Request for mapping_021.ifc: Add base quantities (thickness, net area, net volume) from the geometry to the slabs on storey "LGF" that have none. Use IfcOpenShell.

First a look at what the model holds.

```python
import ifcopenshell
import ifcopenshell.util.element
import ifcopenshell.util.unit

model = ifcopenshell.open("mapping_021.ifc")
print(model.schema)
for unit_type in ("LENGTHUNIT", "AREAUNIT", "VOLUMEUNIT"):
    print(unit_type, ifcopenshell.util.unit.calculate_unit_scale(model, unit_type))
storey = next(s for s in model.by_type("IfcBuildingStorey") if s.Name == "LGF")
slabs = [e for e in ifcopenshell.util.element.get_decomposition(storey) if e.is_a("IfcSlab")]
for e in sorted(slabs, key=lambda e: e.id()):
    print(e.id(), e.is_a(), e.Name, list(ifcopenshell.util.element.get_psets(e, qtos_only=True)), sep=" | ")
```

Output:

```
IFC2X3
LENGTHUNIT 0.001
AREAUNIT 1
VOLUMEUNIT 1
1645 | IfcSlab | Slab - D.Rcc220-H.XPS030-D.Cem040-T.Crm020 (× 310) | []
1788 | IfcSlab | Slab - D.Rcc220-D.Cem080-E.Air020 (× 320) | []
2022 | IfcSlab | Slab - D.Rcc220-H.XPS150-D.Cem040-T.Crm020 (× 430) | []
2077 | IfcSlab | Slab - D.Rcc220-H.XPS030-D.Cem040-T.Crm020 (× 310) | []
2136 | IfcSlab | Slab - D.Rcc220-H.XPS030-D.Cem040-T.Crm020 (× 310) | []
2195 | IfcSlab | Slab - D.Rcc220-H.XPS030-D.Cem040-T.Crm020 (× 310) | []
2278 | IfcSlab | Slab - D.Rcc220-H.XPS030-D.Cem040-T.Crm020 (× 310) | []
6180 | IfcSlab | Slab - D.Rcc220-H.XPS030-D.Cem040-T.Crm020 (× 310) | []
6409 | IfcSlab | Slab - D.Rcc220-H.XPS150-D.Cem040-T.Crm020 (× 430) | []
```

```python
import ifcopenshell
import ifcopenshell.api.pset
import ifcopenshell.geom
import ifcopenshell.util.element
import ifcopenshell.util.shape
import ifcopenshell.util.unit

model = ifcopenshell.open("mapping_021.ifc")
unit_scale = ifcopenshell.util.unit.calculate_unit_scale(model)
area_scale = ifcopenshell.util.unit.calculate_unit_scale(model, "AREAUNIT")
volume_scale = ifcopenshell.util.unit.calculate_unit_scale(model, "VOLUMEUNIT")
settings = ifcopenshell.geom.settings()

storey = next(s for s in model.by_type("IfcBuildingStorey") if s.Name == "LGF")
slabs = [e for e in ifcopenshell.util.element.get_decomposition(storey) if e.is_a("IfcSlab")]

for e in sorted(slabs, key=lambda e: e.id()):
    if ifcopenshell.util.element.get_psets(e, qtos_only=True, should_inherit=False):
        continue
    # Geometry comes back in metres, in the element's own axes.
    shape = ifcopenshell.geom.create_shape(settings, e)
    values = {
        "Width": ifcopenshell.util.shape.get_z(shape.geometry) / unit_scale,
        "NetArea": ifcopenshell.util.shape.get_footprint_area(shape.geometry) / area_scale,
        "NetVolume": ifcopenshell.util.shape.get_volume(shape.geometry) / volume_scale,
    }
    qto = ifcopenshell.api.pset.add_qto(model, product=e, name="BaseQuantities")
    ifcopenshell.api.pset.edit_qto(model, qto=qto, properties=values)
    print(e.id(), {k: round(v, 3) for k, v in values.items()})

model.write("mapping_021_edited.ifc")
```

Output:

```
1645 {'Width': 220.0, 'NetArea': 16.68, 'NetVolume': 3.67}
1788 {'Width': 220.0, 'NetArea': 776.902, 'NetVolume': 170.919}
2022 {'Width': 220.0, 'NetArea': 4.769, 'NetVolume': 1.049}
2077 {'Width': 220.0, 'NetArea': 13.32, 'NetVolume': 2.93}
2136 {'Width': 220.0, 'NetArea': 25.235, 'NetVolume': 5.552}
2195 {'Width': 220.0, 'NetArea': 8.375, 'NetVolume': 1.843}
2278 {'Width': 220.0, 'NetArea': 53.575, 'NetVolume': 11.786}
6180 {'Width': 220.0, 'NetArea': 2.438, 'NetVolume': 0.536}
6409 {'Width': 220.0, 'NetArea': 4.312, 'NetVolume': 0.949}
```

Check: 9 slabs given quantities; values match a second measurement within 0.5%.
